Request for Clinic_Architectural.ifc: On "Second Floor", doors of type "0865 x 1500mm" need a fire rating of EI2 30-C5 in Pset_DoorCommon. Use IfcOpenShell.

First a look at what the model holds.

```python
import ifcopenshell
import ifcopenshell.util.element

model = ifcopenshell.open("Clinic_Architectural.ifc")
print(model.schema)
storey = next(s for s in model.by_type("IfcBuildingStorey") if s.Name == "Second Floor")
doors = [e for e in ifcopenshell.util.element.get_decomposition(storey) if e.is_a("IfcDoor")]
seen = {}
for e in doors:
    element_type = ifcopenshell.util.element.get_type(e)
    key = (element_type.Name if element_type != e and element_type else None, ifcopenshell.util.element.get_pset(e, "Pset_DoorCommon", "FireRating"))
    seen[key] = seen.get(key, 0) + 1
for (name, value), count in sorted(seen.items(), key=str):
    print(count, "x", name, "|", value)
```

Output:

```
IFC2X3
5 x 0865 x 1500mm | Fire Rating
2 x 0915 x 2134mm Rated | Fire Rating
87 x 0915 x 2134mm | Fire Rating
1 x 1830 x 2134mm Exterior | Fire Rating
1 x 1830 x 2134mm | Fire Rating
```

```python
import ifcopenshell
import ifcopenshell.api.pset
import ifcopenshell.util.element

model = ifcopenshell.open("Clinic_Architectural.ifc")

storey = next(s for s in model.by_type("IfcBuildingStorey") if s.Name == "Second Floor")
doors = [e for e in ifcopenshell.util.element.get_decomposition(storey) if e.is_a("IfcDoor")]

count = 0
for e in doors:
    element_type = ifcopenshell.util.element.get_type(e)
    if element_type in (None, e) or element_type.Name != "0865 x 1500mm":
        continue
    # add_pset returns the element's existing set when there is one.
    pset = ifcopenshell.api.pset.add_pset(model, product=e, name="Pset_DoorCommon")
    ifcopenshell.api.pset.edit_pset(model, pset=pset, properties={"FireRating": "EI2 30-C5"})
    count += 1

print(count, "doors updated")

model.write("Clinic_Architectural_updated.ifc")
```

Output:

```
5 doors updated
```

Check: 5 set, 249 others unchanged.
